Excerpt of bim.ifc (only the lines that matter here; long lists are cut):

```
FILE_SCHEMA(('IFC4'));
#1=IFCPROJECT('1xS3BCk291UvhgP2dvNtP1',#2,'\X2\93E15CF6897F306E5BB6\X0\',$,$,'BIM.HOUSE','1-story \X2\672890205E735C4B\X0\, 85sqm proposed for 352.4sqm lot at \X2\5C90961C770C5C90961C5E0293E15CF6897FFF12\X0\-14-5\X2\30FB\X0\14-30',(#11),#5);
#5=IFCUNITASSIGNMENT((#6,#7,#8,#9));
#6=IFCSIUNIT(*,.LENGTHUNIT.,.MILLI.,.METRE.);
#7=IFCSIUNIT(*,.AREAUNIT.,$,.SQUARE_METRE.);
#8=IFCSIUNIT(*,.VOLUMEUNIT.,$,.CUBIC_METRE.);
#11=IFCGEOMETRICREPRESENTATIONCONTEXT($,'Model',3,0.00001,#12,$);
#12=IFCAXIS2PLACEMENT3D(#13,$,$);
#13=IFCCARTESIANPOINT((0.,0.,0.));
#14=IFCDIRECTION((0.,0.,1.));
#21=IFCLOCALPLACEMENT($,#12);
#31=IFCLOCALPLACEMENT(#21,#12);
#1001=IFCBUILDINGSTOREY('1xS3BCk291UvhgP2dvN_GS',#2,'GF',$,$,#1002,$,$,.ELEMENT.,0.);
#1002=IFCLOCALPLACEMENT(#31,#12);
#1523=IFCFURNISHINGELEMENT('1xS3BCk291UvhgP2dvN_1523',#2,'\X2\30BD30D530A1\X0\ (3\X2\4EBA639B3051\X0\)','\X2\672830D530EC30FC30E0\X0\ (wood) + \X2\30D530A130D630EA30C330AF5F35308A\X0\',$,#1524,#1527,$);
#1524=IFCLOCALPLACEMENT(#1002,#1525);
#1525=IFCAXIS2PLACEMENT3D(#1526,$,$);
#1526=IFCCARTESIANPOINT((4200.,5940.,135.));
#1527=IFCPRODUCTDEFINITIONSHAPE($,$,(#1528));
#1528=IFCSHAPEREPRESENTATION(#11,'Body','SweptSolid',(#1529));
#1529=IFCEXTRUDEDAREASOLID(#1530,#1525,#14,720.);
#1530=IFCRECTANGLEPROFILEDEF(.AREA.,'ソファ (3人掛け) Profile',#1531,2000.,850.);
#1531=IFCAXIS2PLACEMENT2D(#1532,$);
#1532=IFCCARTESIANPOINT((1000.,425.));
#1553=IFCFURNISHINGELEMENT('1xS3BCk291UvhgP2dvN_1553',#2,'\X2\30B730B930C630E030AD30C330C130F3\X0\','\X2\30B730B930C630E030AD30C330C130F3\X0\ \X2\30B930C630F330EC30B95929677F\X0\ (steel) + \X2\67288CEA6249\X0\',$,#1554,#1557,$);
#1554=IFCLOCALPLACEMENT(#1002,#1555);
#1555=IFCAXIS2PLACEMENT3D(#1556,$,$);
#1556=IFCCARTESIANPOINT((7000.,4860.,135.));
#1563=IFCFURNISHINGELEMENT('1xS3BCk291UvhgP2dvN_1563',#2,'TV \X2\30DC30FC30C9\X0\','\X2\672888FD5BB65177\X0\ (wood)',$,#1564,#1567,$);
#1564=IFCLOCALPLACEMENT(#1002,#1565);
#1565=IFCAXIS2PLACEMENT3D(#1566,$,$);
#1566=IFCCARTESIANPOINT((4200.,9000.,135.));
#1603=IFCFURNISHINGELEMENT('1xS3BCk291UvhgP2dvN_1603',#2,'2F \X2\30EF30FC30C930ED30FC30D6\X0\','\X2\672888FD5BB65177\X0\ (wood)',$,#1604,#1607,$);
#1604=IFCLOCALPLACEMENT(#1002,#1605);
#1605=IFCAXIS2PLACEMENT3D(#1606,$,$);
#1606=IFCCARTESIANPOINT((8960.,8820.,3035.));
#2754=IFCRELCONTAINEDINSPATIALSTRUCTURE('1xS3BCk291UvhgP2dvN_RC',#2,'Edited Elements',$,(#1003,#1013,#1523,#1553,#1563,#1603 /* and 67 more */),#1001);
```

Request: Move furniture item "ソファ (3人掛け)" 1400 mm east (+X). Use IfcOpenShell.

```python
import ifcopenshell
import ifcopenshell.api.geometry
import ifcopenshell.util.placement

model = ifcopenshell.open("bim.ifc")

item = model.by_guid("1xS3BCk291UvhgP2dvN_1523")
matrix = ifcopenshell.util.placement.get_local_placement(item.ObjectPlacement)
matrix[0, 3] += 1400.0
ifcopenshell.api.geometry.edit_object_placement(model, product=item, matrix=matrix, is_si=False)

print(ifcopenshell.util.placement.get_local_placement(item.ObjectPlacement).round(3) + 0.0)

model.write("bim_edited.ifc")
```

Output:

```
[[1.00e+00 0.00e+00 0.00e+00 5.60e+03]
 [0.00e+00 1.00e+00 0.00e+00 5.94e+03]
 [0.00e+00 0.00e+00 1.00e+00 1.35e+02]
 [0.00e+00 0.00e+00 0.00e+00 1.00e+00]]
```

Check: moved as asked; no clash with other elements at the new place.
